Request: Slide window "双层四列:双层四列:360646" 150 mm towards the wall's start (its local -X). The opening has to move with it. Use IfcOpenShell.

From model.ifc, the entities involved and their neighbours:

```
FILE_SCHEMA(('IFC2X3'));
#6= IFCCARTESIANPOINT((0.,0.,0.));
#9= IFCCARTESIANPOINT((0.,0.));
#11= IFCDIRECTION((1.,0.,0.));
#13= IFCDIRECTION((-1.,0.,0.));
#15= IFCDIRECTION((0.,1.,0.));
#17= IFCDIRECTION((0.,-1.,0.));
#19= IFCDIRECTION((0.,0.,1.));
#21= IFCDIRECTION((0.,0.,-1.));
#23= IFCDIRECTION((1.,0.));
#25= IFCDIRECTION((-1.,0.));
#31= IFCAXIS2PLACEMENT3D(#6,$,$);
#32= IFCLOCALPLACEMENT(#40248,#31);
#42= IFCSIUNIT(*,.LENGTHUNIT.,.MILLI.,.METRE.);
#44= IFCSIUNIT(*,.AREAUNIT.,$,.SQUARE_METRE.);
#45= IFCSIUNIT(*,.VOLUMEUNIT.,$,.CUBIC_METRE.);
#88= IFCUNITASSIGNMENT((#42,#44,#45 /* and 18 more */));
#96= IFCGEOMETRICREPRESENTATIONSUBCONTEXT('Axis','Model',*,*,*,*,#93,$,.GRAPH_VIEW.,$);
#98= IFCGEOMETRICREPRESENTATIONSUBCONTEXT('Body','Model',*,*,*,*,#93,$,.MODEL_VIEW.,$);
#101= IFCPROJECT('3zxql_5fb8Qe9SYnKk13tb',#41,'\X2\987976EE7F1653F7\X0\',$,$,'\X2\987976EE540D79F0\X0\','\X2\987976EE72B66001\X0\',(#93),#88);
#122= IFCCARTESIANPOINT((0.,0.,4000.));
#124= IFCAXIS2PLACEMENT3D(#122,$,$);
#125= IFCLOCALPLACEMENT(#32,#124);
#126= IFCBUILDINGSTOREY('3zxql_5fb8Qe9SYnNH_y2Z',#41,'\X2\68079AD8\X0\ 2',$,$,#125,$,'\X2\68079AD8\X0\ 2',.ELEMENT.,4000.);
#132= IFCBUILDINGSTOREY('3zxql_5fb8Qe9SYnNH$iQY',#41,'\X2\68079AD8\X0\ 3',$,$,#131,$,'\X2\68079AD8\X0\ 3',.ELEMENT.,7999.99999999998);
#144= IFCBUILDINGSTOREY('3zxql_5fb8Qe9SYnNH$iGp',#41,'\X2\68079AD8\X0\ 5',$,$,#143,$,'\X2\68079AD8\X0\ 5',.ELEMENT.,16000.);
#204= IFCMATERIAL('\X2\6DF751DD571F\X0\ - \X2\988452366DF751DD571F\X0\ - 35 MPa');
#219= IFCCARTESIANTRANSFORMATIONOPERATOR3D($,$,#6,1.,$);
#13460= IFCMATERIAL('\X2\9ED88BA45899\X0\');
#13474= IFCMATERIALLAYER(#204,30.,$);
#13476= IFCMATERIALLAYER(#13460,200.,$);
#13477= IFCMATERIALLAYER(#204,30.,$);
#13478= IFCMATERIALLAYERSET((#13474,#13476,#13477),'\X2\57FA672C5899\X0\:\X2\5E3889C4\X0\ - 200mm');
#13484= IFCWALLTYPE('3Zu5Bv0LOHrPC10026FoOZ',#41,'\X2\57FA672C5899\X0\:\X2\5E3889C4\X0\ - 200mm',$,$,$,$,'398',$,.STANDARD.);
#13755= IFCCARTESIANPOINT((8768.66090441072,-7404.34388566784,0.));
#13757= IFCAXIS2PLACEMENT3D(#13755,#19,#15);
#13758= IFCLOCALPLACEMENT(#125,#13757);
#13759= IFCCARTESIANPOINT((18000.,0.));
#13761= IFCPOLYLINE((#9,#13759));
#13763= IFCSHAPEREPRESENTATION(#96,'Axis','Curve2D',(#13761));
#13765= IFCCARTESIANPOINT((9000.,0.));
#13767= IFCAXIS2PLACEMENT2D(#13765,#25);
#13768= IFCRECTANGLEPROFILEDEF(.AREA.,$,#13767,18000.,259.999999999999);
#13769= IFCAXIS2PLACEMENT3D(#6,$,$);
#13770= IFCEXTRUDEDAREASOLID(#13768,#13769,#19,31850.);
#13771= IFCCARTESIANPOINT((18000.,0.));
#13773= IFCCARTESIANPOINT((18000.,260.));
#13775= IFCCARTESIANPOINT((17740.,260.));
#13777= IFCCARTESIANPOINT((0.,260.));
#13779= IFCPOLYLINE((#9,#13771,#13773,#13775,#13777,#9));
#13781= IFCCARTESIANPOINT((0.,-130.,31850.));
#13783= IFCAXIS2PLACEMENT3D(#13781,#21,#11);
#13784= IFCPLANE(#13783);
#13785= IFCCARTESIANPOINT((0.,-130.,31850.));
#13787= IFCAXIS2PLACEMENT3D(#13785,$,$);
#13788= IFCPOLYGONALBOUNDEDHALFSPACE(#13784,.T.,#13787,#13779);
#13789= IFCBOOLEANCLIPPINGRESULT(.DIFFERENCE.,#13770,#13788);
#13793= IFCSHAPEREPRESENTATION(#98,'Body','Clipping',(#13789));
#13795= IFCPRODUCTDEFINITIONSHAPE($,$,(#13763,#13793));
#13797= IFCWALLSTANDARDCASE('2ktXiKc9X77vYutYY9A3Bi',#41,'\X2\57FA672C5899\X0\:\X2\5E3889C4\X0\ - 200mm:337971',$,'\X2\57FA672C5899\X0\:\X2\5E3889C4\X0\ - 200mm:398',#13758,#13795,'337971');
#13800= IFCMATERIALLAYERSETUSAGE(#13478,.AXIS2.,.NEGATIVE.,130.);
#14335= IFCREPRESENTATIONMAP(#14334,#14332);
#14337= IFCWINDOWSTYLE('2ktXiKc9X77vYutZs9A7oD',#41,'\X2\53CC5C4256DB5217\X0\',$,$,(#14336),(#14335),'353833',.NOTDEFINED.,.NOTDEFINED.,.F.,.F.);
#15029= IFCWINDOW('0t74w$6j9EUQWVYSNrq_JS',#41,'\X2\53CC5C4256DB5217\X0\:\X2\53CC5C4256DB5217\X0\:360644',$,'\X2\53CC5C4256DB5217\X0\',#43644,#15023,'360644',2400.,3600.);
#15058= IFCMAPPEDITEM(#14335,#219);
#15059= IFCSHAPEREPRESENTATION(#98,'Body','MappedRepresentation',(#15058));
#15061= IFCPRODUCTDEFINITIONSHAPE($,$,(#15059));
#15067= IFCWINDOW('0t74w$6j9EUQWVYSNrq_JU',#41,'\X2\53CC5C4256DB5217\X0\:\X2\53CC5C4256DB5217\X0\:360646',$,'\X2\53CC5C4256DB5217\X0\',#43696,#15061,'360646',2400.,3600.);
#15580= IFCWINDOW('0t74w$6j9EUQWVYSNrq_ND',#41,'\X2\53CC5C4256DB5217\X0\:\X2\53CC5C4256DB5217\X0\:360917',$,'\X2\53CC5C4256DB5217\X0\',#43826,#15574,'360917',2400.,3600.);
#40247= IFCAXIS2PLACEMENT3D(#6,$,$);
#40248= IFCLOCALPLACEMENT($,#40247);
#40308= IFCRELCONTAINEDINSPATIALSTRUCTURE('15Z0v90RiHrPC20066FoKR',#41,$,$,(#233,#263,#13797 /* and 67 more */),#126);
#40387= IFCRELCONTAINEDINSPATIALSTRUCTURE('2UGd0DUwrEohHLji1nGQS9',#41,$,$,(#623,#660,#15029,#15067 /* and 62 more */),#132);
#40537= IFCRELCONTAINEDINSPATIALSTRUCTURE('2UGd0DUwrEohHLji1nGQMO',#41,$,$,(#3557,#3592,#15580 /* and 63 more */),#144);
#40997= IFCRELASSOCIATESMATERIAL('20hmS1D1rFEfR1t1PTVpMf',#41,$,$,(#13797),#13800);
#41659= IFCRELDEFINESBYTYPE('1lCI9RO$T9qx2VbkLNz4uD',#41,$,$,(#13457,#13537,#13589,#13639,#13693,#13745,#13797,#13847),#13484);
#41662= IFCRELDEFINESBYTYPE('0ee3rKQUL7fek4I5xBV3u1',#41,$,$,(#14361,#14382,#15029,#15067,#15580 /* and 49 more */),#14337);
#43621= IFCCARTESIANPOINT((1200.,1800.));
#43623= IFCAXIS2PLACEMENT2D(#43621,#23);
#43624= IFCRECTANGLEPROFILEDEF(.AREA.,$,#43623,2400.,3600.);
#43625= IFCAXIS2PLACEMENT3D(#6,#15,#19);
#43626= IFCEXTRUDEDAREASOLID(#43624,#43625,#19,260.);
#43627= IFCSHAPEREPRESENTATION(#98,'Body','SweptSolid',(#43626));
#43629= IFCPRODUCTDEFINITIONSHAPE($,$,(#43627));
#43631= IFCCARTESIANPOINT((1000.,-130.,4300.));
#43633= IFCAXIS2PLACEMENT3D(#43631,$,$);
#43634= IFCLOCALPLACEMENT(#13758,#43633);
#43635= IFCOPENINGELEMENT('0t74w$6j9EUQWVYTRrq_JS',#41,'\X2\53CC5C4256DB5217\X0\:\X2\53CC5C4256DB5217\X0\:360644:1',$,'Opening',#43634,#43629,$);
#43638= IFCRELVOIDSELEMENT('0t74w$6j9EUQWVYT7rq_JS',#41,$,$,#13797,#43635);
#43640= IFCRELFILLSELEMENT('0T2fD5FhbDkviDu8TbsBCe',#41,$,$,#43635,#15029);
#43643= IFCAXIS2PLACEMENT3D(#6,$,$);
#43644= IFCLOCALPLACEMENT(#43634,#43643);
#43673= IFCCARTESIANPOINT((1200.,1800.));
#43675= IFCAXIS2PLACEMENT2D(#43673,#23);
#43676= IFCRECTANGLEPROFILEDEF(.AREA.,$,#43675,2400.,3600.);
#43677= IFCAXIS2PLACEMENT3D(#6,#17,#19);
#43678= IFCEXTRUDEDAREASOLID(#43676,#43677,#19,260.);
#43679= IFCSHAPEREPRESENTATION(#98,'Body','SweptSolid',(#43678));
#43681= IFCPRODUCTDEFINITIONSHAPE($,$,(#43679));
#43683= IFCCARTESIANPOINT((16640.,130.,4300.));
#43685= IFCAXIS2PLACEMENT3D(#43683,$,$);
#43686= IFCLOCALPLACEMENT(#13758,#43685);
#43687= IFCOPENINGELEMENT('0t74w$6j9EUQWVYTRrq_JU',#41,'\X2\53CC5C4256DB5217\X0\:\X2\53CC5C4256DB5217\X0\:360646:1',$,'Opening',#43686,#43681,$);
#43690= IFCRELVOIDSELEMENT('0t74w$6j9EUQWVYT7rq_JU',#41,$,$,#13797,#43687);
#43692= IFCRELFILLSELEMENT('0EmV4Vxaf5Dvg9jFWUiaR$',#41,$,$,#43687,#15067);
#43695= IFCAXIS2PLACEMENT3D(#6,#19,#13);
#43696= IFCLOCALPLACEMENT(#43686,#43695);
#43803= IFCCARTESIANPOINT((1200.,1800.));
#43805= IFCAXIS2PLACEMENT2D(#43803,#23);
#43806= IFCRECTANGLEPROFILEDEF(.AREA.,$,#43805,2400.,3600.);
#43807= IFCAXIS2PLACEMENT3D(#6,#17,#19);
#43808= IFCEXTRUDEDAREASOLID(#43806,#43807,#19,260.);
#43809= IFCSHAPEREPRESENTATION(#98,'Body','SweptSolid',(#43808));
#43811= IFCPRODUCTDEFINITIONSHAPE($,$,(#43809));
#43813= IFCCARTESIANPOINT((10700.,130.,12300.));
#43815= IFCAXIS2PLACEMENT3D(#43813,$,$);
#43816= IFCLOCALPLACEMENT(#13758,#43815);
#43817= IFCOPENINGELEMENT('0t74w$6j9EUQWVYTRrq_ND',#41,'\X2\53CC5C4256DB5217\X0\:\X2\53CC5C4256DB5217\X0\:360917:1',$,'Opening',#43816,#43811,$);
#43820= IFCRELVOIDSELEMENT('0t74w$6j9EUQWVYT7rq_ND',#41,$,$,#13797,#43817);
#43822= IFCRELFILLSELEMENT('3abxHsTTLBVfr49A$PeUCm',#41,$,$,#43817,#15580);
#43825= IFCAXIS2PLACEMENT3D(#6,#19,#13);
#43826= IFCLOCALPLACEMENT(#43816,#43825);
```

```python
import ifcopenshell
import ifcopenshell.api.geometry
import ifcopenshell.util.placement

model = ifcopenshell.open("model.ifc")

window = model.by_guid("0t74w$6j9EUQWVYSNrq_JU")
opening = window.FillsVoids[0].RelatingOpeningElement
wall = opening.VoidsElements[0].RelatingBuildingElement

wall_matrix = ifcopenshell.util.placement.get_local_placement(wall.ObjectPlacement)
shift = wall_matrix[:3, 0] * -150.0
before = ifcopenshell.util.placement.get_local_placement(window.ObjectPlacement)[:3, 3].copy()

# The window is placed relative to its opening, so it follows when the opening moves.
matrix = ifcopenshell.util.placement.get_local_placement(opening.ObjectPlacement)
matrix[:3, 3] += shift
ifcopenshell.api.geometry.edit_object_placement(
    model, product=opening, matrix=matrix, is_si=False, should_transform_children=True
)

after = ifcopenshell.util.placement.get_local_placement(window.ObjectPlacement)[:3, 3]
print("window moved by", (after - before).round(3) + 0.0)

model.write("model_edited.ifc")
```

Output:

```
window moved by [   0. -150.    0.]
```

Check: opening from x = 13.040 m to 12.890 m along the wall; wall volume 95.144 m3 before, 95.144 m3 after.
